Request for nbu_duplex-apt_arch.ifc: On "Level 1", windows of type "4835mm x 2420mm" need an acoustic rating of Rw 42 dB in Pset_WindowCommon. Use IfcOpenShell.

First a look at what the model holds.

```python
import ifcopenshell
import ifcopenshell.util.element

model = ifcopenshell.open("nbu_duplex-apt_arch.ifc")
print(model.schema)
storey = next(s for s in model.by_type("IfcBuildingStorey") if s.Name == "Level 1")
windows = [e for e in ifcopenshell.util.element.get_decomposition(storey) if e.is_a("IfcWindow")]
seen = {}
for e in windows:
    element_type = ifcopenshell.util.element.get_type(e)
    key = (element_type.Name if element_type != e and element_type else None, ifcopenshell.util.element.get_pset(e, "Pset_WindowCommon", "AcousticRating"))
    seen[key] = seen.get(key, 0) + 1
for (name, value), count in sorted(seen.items(), key=str):
    print(count, "x", name, "|", value)
```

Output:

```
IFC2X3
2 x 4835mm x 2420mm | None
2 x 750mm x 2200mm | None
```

```python
import ifcopenshell
import ifcopenshell.api.pset
import ifcopenshell.util.element

model = ifcopenshell.open("nbu_duplex-apt_arch.ifc")

storey = next(s for s in model.by_type("IfcBuildingStorey") if s.Name == "Level 1")
windows = [e for e in ifcopenshell.util.element.get_decomposition(storey) if e.is_a("IfcWindow")]

count = 0
for e in windows:
    element_type = ifcopenshell.util.element.get_type(e)
    if element_type in (None, e) or element_type.Name != "4835mm x 2420mm":
        continue
    # add_pset returns the element's existing set when there is one.
    pset = ifcopenshell.api.pset.add_pset(model, product=e, name="Pset_WindowCommon")
    ifcopenshell.api.pset.edit_pset(model, pset=pset, properties={"AcousticRating": "Rw 42 dB"})
    count += 1

print(count, "windows updated")

model.write("nbu_duplex-apt_arch_updated.ifc")
```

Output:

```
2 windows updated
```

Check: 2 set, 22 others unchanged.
